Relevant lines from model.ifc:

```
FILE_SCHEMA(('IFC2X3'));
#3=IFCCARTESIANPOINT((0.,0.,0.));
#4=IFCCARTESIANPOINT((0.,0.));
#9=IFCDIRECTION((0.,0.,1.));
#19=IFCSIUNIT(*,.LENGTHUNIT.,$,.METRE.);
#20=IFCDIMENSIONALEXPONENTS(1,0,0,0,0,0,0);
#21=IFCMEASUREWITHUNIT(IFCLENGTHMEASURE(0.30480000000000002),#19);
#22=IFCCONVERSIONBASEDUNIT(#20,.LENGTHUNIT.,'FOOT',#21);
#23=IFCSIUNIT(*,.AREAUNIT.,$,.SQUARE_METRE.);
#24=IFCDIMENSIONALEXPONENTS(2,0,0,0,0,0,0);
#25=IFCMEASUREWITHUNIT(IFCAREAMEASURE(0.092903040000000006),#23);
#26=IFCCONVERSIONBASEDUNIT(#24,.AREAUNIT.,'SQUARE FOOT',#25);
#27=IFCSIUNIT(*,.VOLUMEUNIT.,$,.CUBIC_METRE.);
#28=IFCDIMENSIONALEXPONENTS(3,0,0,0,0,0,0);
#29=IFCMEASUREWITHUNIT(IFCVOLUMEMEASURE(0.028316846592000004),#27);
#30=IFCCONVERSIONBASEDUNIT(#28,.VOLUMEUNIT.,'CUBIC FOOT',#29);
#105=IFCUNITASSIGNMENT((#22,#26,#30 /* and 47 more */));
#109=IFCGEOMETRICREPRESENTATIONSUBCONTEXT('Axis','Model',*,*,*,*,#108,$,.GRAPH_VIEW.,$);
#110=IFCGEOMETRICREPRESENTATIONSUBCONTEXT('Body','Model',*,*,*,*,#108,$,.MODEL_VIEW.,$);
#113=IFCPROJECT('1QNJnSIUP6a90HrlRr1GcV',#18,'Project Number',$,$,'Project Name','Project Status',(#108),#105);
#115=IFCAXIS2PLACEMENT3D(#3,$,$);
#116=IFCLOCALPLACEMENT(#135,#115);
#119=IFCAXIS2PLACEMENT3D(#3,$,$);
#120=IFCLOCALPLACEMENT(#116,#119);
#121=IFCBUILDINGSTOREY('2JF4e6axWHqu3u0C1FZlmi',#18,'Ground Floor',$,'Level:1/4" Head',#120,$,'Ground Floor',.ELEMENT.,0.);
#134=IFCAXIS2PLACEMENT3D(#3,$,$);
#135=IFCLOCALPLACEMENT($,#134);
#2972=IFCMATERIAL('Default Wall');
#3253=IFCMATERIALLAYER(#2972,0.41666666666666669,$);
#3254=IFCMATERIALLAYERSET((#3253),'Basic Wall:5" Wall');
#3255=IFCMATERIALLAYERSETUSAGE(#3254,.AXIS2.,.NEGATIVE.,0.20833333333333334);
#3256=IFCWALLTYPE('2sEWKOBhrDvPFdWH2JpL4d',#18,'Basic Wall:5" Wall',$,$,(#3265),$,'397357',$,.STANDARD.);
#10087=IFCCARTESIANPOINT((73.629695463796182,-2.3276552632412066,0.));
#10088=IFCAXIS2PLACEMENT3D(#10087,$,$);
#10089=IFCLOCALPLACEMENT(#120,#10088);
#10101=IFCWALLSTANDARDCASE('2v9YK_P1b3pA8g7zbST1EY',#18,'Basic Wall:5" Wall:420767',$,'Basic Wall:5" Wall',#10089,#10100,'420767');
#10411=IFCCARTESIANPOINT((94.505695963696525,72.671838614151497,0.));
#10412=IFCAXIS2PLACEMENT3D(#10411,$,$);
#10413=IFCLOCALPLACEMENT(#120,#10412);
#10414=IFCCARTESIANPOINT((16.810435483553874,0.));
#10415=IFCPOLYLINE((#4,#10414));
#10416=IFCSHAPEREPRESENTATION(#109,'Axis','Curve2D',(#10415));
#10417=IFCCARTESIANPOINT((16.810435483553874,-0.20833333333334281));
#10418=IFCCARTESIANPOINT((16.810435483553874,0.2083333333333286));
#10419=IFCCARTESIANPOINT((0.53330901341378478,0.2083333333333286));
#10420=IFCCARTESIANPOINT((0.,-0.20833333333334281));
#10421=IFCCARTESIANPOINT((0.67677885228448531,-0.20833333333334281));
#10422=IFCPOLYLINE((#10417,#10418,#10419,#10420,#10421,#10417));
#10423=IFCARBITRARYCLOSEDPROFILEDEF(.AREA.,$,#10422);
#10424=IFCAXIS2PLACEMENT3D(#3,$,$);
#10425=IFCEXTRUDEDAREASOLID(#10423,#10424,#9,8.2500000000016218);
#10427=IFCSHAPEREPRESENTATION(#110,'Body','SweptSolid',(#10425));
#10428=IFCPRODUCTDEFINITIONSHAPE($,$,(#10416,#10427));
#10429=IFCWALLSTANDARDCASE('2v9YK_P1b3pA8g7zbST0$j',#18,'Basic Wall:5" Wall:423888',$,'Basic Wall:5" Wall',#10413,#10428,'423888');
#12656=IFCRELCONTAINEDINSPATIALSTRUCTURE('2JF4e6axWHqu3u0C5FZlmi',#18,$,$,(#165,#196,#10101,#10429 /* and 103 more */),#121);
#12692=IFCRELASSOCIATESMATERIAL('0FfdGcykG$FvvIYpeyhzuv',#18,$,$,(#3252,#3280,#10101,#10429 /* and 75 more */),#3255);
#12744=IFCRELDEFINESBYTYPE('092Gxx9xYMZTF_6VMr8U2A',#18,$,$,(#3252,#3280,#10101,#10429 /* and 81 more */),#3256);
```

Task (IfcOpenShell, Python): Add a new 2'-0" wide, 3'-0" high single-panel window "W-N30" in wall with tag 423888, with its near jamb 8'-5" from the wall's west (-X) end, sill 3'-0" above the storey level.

```python
import numpy as np
import ifcopenshell
import ifcopenshell.api.feature
import ifcopenshell.api.geometry
import ifcopenshell.api.root
import ifcopenshell.api.spatial
import ifcopenshell.api.type
import ifcopenshell.geom
import ifcopenshell.util.element
import ifcopenshell.util.placement
import ifcopenshell.util.representation
import ifcopenshell.util.shape
import ifcopenshell.util.unit

model = ifcopenshell.open("model.ifc")
unit_scale = ifcopenshell.util.unit.calculate_unit_scale(model)
settings = ifcopenshell.geom.settings()


def volume(element):
    """Net volume in cubic metres, openings subtracted."""
    shape = ifcopenshell.geom.create_shape(settings, element)
    return ifcopenshell.util.shape.get_volume(shape.geometry)


wall = model.by_guid("2v9YK_P1b3pA8g7zbST0$j")
storey = ifcopenshell.util.element.get_container(wall, ifc_class="IfcBuildingStorey")
context = ifcopenshell.util.representation.get_context(model, "Model", "Body", "MODEL_VIEW")
before = volume(wall)

width, height, from_end, sill = 0.6096, 0.9144, 2.5654, 0.9144  # metres

# The wall runs along its own X axis, and the end named is its -X end.
wall_shape = ifcopenshell.geom.create_shape(settings, wall)
x, y, z = ifcopenshell.util.shape.get_vertices(wall_shape.geometry).T
start = x.min() + from_end
face, thickness = float(y.min()), float(y.max() - y.min())
wall_matrix = ifcopenshell.util.placement.get_local_placement(wall.ObjectPlacement)
level = ifcopenshell.util.placement.get_local_placement(storey.ObjectPlacement)[2, 3]


def in_wall(x, y):
    """Placement at x, y metres in the wall's axes, at sill height."""
    matrix = wall_matrix.copy()
    matrix[:, 3] = wall_matrix @ np.array([x / unit_scale, y / unit_scale, 0.0, 1.0])
    matrix[2, 3] = level + sill / unit_scale
    return matrix


# Opening: a box that overshoots both wall faces by 50 mm.
opening = ifcopenshell.api.root.create_entity(model, ifc_class="IfcOpeningElement")
box = ifcopenshell.api.geometry.add_wall_representation(
    model, context=context, length=width, height=height, thickness=thickness + 0.1
)
ifcopenshell.api.geometry.assign_representation(model, product=opening, representation=box)
ifcopenshell.api.geometry.edit_object_placement(model, product=opening, matrix=in_wall(start, face - 0.05), is_si=False)
ifcopenshell.api.feature.add_feature(model, feature=opening, element=wall)

window = ifcopenshell.api.root.create_entity(model, ifc_class="IfcWindow", name="W-N30")
window.OverallWidth, window.OverallHeight = width / unit_scale, height / unit_scale
body = ifcopenshell.api.geometry.add_window_representation(
    model,
    context=context,
    overall_width=window.OverallWidth,
    overall_height=window.OverallHeight,
    partition_type="SINGLE_PANEL",
)
ifcopenshell.api.geometry.assign_representation(model, product=window, representation=body)
ifcopenshell.api.spatial.assign_container(model, products=[window], relating_structure=storey)
fills = ifcopenshell.api.feature.add_filling(model, opening=opening, element=window)
fills.OwnerHistory = window.OwnerHistory  # required in IFC2X3

# IFC2X3 keeps the operation on the window style.
style = ifcopenshell.api.root.create_entity(model, ifc_class="IfcWindowStyle", name="W-N30")
style.OperationType, style.ConstructionType = "SINGLE_PANEL", "NOTDEFINED"
style.ParameterTakesPrecedence = style.Sizeable = False
ifcopenshell.api.type.assign_type(model, related_objects=[window], relating_type=style)

# Centre the window in the wall's thickness.
ifcopenshell.api.geometry.edit_object_placement(model, product=window, matrix=in_wall(start, face), is_si=False)
window_shape = ifcopenshell.geom.create_shape(settings, window)
depth = ifcopenshell.util.shape.get_vertices(window_shape.geometry)[:, 1]
offset = face + thickness / 2 - (depth.min() + depth.max()) / 2
ifcopenshell.api.geometry.edit_object_placement(model, product=window, matrix=in_wall(start, offset), is_si=False)

after = volume(wall)

print(f"wall volume {before:.3f} -> {after:.3f} m3")

model.write("model-out.ifc")
```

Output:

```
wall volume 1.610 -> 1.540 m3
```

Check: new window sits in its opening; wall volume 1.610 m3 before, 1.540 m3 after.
